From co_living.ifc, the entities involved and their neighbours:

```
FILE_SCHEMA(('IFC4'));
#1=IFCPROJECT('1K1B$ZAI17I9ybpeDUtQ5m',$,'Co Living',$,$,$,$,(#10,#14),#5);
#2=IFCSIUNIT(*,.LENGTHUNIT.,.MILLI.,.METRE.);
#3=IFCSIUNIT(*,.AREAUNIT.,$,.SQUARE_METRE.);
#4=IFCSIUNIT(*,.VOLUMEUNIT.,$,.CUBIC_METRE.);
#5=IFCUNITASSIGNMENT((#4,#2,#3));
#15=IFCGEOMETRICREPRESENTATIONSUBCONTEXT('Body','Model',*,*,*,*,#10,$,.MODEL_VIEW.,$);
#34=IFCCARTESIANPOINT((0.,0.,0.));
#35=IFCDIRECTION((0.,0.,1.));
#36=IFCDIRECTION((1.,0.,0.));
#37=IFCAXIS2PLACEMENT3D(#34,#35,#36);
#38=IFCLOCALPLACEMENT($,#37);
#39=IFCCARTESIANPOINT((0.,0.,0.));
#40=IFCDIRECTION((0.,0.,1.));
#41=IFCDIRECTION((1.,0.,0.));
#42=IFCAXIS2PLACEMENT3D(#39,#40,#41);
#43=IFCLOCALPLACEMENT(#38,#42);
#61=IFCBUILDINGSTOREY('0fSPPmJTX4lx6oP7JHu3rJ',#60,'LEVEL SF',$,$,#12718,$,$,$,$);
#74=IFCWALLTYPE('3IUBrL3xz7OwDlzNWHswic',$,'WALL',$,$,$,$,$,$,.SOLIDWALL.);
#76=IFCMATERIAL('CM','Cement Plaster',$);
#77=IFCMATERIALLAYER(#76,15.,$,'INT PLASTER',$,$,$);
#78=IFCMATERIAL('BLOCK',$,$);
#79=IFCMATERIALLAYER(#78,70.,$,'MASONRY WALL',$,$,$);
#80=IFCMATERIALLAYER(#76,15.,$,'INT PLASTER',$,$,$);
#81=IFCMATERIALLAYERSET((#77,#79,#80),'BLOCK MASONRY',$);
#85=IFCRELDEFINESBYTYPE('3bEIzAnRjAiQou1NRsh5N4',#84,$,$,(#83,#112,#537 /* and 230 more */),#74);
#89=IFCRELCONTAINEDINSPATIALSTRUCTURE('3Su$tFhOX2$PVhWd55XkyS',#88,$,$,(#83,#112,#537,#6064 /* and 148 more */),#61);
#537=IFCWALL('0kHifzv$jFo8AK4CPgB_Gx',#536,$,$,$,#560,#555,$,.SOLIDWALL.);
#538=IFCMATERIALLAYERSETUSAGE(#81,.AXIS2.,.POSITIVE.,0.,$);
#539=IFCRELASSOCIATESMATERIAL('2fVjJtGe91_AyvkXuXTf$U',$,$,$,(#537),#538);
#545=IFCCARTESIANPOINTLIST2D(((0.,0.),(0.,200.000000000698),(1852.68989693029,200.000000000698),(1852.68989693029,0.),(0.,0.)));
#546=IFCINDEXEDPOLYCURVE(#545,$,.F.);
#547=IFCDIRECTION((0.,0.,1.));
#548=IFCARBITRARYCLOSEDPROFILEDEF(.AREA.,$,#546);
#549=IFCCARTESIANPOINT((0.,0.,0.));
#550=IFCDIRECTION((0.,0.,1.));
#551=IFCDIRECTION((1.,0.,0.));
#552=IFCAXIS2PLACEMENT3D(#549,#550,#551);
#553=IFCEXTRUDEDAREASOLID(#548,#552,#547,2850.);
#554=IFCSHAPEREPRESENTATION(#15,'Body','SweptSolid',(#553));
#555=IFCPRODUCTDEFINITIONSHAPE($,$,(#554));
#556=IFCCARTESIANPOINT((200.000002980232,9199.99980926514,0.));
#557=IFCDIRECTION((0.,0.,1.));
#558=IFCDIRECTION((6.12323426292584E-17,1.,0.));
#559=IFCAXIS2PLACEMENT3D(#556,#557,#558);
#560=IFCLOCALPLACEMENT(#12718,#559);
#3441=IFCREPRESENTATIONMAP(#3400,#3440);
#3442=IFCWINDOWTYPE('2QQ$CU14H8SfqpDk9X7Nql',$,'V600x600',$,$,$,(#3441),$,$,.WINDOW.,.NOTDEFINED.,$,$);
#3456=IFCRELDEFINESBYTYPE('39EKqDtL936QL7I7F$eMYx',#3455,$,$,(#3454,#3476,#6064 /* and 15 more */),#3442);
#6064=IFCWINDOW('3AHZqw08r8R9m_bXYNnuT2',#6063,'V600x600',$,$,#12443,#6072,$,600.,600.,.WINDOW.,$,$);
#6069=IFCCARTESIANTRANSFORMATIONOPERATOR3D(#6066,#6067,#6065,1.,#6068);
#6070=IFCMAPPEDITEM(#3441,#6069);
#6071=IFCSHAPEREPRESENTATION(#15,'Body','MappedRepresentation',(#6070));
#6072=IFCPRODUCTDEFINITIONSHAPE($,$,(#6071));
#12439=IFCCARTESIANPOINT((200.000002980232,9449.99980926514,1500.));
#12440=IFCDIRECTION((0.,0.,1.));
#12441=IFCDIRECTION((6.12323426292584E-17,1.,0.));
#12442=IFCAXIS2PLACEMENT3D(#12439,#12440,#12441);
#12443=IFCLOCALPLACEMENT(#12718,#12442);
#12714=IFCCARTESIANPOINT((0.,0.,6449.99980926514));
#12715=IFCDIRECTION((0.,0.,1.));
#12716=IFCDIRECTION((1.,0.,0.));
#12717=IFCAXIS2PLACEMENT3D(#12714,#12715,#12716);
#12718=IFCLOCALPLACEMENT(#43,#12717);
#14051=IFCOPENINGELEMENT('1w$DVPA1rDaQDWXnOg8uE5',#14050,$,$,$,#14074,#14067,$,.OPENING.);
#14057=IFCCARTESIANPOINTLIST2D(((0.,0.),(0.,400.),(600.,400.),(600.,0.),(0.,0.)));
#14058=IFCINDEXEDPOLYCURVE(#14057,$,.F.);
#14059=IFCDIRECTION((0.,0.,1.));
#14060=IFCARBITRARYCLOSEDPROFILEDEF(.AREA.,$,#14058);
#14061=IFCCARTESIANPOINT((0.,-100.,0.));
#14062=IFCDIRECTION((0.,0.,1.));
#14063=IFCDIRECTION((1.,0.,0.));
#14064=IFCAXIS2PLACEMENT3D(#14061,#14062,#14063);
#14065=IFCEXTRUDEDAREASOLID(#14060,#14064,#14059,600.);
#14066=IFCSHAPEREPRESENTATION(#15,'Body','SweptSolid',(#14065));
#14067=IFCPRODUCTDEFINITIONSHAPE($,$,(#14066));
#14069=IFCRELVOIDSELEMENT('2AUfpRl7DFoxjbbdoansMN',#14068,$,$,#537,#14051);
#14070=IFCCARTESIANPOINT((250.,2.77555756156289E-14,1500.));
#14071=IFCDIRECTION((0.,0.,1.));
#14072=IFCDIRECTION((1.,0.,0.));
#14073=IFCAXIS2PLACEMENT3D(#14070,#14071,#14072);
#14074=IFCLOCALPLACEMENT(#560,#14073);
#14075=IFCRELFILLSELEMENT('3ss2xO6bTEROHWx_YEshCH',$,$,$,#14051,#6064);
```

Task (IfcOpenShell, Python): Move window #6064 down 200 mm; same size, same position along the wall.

```python
import numpy as np
import ifcopenshell
import ifcopenshell.api.geometry
import ifcopenshell.util.placement
import ifcopenshell.util.unit

model = ifcopenshell.open("co_living.ifc")
unit_scale = ifcopenshell.util.unit.calculate_unit_scale(model)

window = model.by_id(6064)
opening = window.FillsVoids[0].RelatingOpeningElement
dz = -200.0

shift = np.array([0.0, 0.0, dz])
# The window is not placed relative to its opening, so move both.
for product in (opening, window):
    matrix = ifcopenshell.util.placement.get_local_placement(product.ObjectPlacement)
    matrix[:3, 3] += shift
    ifcopenshell.api.geometry.edit_object_placement(model, product=product, matrix=matrix, is_si=False)

print(f"moved by {dz * unit_scale:+.3f} m")

model.write("co_living_v2.ifc")
```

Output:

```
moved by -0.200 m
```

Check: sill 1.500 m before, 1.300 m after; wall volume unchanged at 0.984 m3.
